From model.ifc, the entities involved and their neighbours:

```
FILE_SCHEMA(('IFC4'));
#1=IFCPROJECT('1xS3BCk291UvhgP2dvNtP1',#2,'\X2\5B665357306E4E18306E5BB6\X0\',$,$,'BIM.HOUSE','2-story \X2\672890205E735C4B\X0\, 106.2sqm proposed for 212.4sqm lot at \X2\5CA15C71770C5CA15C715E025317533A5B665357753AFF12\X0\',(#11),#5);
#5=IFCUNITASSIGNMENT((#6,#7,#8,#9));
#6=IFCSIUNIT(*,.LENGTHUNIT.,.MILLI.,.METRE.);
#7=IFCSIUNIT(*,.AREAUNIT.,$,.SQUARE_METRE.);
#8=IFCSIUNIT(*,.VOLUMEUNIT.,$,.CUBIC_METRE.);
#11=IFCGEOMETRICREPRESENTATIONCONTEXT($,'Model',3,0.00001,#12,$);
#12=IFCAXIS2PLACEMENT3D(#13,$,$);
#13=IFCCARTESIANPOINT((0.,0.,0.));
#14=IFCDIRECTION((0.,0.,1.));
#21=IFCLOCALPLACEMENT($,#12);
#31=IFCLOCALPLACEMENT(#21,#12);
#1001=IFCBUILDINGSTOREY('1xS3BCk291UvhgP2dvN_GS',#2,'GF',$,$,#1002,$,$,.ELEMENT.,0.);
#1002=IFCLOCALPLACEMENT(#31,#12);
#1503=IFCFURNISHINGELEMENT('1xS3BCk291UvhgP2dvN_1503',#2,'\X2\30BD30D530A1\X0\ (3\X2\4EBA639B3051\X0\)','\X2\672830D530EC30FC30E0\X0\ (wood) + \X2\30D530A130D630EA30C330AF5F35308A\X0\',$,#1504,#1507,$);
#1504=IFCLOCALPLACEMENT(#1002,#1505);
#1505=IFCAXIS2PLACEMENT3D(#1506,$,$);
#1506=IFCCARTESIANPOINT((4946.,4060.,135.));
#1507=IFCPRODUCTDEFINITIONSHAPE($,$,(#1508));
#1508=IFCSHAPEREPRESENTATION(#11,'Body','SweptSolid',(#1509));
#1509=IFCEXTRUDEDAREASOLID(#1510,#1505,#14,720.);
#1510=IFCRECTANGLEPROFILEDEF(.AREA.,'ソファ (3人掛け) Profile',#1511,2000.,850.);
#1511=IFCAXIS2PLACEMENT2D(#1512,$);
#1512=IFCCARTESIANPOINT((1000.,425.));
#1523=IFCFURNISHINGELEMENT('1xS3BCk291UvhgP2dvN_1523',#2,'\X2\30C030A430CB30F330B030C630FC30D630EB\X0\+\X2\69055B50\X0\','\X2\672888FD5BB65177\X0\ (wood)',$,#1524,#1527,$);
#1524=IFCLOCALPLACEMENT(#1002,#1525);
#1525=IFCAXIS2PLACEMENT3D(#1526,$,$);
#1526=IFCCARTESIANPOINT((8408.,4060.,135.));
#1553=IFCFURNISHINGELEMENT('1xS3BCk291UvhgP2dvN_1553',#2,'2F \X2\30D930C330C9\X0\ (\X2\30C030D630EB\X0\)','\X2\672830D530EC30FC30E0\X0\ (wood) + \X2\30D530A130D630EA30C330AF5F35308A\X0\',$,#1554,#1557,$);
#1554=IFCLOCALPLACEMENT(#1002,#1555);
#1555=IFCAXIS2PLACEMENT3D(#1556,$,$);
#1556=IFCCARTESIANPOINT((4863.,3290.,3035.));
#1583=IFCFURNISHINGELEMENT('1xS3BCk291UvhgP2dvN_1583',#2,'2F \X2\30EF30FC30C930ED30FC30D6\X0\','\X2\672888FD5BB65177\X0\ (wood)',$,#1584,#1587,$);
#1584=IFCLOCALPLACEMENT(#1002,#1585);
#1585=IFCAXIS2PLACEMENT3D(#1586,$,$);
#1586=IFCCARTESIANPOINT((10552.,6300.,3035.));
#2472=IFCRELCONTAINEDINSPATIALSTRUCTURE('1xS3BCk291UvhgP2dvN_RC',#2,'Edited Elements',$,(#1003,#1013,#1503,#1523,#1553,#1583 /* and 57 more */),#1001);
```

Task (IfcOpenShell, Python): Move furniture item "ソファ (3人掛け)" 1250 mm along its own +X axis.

```python
import ifcopenshell
import ifcopenshell.api.geometry
import ifcopenshell.util.placement

model = ifcopenshell.open("model.ifc")

item = model.by_guid("1xS3BCk291UvhgP2dvN_1503")
matrix = ifcopenshell.util.placement.get_local_placement(item.ObjectPlacement)
matrix[:3, 3] += matrix[:3, 0] * 1250.0
ifcopenshell.api.geometry.edit_object_placement(model, product=item, matrix=matrix, is_si=False)

print(ifcopenshell.util.placement.get_local_placement(item.ObjectPlacement).round(3) + 0.0)

model.write("model_updated.ifc")
```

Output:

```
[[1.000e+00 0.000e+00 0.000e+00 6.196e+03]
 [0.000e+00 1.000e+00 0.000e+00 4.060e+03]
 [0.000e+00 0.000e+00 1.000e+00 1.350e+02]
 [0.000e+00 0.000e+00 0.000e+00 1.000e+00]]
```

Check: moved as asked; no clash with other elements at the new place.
